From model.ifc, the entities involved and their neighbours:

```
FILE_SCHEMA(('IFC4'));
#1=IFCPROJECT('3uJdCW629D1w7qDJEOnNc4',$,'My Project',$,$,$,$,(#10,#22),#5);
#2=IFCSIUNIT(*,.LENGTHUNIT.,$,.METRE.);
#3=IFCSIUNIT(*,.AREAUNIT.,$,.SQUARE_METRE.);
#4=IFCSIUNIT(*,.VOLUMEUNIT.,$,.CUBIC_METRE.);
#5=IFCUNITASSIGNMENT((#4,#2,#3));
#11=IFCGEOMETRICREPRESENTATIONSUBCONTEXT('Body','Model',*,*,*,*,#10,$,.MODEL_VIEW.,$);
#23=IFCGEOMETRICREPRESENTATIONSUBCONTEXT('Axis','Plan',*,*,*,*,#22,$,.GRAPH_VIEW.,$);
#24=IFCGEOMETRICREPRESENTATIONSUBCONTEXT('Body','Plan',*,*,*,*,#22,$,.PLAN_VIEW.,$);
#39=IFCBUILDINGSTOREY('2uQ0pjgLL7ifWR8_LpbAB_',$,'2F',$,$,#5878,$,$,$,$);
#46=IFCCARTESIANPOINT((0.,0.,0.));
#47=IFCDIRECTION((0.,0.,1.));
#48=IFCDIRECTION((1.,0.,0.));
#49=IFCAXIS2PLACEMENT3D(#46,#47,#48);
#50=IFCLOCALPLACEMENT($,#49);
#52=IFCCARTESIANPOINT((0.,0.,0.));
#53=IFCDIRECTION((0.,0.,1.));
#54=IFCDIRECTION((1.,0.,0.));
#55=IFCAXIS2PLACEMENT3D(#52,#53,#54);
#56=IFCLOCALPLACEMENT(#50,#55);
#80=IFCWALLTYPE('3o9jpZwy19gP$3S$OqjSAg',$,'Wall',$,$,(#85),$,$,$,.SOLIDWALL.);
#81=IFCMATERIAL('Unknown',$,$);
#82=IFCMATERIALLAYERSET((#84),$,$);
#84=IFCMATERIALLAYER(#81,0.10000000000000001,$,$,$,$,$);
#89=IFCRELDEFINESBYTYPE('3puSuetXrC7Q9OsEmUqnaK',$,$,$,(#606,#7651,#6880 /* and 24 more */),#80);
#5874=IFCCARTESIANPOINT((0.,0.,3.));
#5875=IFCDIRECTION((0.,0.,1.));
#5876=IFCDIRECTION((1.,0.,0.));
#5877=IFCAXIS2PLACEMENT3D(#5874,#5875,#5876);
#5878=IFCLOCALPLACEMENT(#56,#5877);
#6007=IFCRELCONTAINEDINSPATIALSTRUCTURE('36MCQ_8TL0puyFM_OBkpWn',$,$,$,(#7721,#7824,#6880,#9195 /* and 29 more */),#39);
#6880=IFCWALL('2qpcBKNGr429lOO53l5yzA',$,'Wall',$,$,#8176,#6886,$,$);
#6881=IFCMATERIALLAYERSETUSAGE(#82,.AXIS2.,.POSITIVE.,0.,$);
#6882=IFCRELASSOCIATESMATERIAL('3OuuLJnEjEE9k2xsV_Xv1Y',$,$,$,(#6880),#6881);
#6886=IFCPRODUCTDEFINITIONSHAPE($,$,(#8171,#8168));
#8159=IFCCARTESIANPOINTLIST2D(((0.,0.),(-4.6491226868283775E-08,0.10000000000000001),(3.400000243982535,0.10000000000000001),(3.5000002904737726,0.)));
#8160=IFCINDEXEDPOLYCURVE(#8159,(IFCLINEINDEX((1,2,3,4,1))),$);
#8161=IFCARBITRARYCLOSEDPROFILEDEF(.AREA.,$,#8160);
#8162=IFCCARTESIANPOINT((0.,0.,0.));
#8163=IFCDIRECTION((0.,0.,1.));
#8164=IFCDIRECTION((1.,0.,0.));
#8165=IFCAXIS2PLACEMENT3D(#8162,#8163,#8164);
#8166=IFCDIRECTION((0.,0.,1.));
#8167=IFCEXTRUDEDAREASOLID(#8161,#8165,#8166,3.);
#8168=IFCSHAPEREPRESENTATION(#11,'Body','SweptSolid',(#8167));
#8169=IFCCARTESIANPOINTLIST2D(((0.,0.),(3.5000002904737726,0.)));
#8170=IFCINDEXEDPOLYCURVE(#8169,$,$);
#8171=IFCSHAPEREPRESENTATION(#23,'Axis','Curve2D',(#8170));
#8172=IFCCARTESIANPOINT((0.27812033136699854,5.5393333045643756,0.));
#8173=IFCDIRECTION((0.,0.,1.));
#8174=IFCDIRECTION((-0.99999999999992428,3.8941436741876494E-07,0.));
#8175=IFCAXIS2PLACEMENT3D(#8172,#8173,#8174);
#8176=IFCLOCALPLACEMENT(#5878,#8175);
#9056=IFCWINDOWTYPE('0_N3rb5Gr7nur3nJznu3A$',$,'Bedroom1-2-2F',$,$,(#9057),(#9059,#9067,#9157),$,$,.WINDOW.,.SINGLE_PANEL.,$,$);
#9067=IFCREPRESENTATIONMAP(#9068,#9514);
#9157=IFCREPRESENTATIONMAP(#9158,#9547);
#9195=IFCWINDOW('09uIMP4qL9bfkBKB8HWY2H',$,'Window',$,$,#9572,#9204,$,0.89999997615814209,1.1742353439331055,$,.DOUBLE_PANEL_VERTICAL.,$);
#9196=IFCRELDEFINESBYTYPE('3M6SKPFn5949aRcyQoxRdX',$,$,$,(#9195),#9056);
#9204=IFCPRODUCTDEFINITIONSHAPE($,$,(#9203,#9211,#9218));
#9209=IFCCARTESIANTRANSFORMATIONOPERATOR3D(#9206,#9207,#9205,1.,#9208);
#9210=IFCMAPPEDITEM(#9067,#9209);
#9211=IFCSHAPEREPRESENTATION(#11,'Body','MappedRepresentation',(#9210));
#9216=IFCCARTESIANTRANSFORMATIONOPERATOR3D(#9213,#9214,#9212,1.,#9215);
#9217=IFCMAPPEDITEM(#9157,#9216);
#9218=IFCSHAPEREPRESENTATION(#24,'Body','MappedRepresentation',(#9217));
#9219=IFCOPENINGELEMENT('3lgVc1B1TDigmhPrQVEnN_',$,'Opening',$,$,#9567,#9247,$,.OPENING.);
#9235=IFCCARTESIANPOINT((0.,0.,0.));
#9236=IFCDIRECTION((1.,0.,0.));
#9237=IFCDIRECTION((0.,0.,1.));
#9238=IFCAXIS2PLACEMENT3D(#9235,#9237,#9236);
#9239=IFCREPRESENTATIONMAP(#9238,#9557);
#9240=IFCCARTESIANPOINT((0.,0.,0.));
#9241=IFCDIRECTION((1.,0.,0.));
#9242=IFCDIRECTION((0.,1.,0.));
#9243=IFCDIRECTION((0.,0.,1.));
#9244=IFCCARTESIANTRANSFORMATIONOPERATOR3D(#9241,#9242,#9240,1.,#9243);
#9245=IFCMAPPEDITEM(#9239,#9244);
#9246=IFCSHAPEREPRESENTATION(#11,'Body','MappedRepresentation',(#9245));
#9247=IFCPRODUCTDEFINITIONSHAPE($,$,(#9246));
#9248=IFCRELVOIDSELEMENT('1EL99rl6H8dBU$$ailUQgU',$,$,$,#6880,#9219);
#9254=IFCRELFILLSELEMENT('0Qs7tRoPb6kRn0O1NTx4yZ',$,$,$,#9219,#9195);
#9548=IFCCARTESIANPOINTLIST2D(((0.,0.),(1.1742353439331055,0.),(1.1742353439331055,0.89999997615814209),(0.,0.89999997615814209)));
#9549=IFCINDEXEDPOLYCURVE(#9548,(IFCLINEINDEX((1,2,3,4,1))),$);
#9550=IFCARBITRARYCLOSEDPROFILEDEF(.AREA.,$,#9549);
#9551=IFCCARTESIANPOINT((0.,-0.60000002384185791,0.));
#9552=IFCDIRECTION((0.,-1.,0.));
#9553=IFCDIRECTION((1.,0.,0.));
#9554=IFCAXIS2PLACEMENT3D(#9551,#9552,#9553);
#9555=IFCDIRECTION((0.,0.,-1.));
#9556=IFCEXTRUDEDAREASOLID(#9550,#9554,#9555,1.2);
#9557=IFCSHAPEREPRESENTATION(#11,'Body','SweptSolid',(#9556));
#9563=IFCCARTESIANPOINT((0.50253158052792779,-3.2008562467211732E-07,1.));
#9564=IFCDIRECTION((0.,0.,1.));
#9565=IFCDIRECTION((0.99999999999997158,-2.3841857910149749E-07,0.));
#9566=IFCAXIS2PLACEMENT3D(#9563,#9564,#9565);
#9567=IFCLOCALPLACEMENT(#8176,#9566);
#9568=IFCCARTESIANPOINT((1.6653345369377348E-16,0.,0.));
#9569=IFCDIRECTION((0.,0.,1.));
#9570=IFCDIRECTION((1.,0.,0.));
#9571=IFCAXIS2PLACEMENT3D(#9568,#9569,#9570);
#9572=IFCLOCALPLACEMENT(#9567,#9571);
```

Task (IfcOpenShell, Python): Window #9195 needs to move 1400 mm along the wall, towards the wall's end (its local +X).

```python
import ifcopenshell
import ifcopenshell.api.geometry
import ifcopenshell.util.placement

model = ifcopenshell.open("model.ifc")

window = model.by_id(9195)
opening = window.FillsVoids[0].RelatingOpeningElement
wall = opening.VoidsElements[0].RelatingBuildingElement

wall_matrix = ifcopenshell.util.placement.get_local_placement(wall.ObjectPlacement)
shift = wall_matrix[:3, 0] * 1.4
before = ifcopenshell.util.placement.get_local_placement(window.ObjectPlacement)[:3, 3].copy()

# The window is placed relative to its opening, so it follows when the opening moves.
matrix = ifcopenshell.util.placement.get_local_placement(opening.ObjectPlacement)
matrix[:3, 3] += shift
ifcopenshell.api.geometry.edit_object_placement(
    model, product=opening, matrix=matrix, is_si=False, should_transform_children=True
)

after = ifcopenshell.util.placement.get_local_placement(window.ObjectPlacement)[:3, 3]
print("window moved by", (after - before).round(3) + 0.0)

model.write("model-out.ifc")
```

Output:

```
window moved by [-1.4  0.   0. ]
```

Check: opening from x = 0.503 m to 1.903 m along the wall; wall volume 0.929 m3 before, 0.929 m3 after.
